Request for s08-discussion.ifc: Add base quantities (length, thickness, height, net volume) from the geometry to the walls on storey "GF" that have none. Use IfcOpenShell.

First a look at what the model holds.

```python
import ifcopenshell
import ifcopenshell.util.element
import ifcopenshell.util.unit

model = ifcopenshell.open("s08-discussion.ifc")
print(model.schema)
for unit_type in ("LENGTHUNIT", "AREAUNIT", "VOLUMEUNIT"):
    print(unit_type, ifcopenshell.util.unit.calculate_unit_scale(model, unit_type))
storey = next(s for s in model.by_type("IfcBuildingStorey") if s.Name == "GF")
walls = [e for e in ifcopenshell.util.element.get_decomposition(storey) if e.is_a("IfcWall")]
for e in sorted(walls, key=lambda e: e.id()):
    print(e.id(), e.is_a(), e.Name, list(ifcopenshell.util.element.get_psets(e, qtos_only=True)), sep=" | ")
```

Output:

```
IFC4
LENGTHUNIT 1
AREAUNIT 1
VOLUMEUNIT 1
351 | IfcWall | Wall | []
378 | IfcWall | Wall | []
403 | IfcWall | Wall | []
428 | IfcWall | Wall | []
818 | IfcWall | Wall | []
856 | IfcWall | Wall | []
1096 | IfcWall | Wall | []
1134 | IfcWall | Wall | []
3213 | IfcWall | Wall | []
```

```python
import ifcopenshell
import ifcopenshell.api.pset
import ifcopenshell.geom
import ifcopenshell.util.element
import ifcopenshell.util.shape
import ifcopenshell.util.unit

model = ifcopenshell.open("s08-discussion.ifc")
unit_scale = ifcopenshell.util.unit.calculate_unit_scale(model)
volume_scale = ifcopenshell.util.unit.calculate_unit_scale(model, "VOLUMEUNIT")
settings = ifcopenshell.geom.settings()

storey = next(s for s in model.by_type("IfcBuildingStorey") if s.Name == "GF")
walls = [e for e in ifcopenshell.util.element.get_decomposition(storey) if e.is_a("IfcWall")]

for e in sorted(walls, key=lambda e: e.id()):
    if ifcopenshell.util.element.get_psets(e, qtos_only=True, should_inherit=False):
        continue
    # Geometry comes back in metres, in the element's own axes.
    shape = ifcopenshell.geom.create_shape(settings, e)
    values = {
        "Length": ifcopenshell.util.shape.get_x(shape.geometry) / unit_scale,
        "Width": ifcopenshell.util.shape.get_y(shape.geometry) / unit_scale,
        "Height": ifcopenshell.util.shape.get_z(shape.geometry) / unit_scale,
        "NetVolume": ifcopenshell.util.shape.get_volume(shape.geometry) / volume_scale,
    }
    qto = ifcopenshell.api.pset.add_qto(model, product=e, name="Qto_WallBaseQuantities")
    ifcopenshell.api.pset.edit_qto(model, qto=qto, properties=values)
    print(e.id(), {k: round(v, 3) for k, v in values.items()})

model.write("s08-discussion_edited.ifc")
```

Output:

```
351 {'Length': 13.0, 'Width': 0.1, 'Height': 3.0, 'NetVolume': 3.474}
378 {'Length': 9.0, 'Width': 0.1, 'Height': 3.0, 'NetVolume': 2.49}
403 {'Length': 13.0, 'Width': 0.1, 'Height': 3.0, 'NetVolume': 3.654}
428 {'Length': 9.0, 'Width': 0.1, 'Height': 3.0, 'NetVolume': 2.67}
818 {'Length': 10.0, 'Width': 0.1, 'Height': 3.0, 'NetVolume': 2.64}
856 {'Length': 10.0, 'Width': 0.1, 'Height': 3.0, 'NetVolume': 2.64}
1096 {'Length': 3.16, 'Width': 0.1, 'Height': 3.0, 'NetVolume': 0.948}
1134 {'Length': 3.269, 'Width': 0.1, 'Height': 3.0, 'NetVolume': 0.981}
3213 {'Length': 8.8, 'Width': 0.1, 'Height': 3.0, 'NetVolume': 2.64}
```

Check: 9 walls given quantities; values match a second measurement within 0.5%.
